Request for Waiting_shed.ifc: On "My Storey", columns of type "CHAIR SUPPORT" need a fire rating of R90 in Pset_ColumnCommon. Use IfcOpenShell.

First a look at what the model holds.

```python
import ifcopenshell
import ifcopenshell.util.element

model = ifcopenshell.open("Waiting_shed.ifc")
print(model.schema)
storey = next(s for s in model.by_type("IfcBuildingStorey") if s.Name == "My Storey")
columns = [e for e in ifcopenshell.util.element.get_decomposition(storey) if e.is_a("IfcColumn")]
seen = {}
for e in columns:
    element_type = ifcopenshell.util.element.get_type(e)
    key = (element_type.Name if element_type != e and element_type else None, ifcopenshell.util.element.get_pset(e, "Pset_ColumnCommon", "FireRating"))
    seen[key] = seen.get(key, 0) + 1
for (name, value), count in sorted(seen.items(), key=str):
    print(count, "x", name, "|", value)
```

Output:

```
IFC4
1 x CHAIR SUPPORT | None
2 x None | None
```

```python
import ifcopenshell
import ifcopenshell.api.pset
import ifcopenshell.util.element

model = ifcopenshell.open("Waiting_shed.ifc")

storey = next(s for s in model.by_type("IfcBuildingStorey") if s.Name == "My Storey")
columns = [e for e in ifcopenshell.util.element.get_decomposition(storey) if e.is_a("IfcColumn")]

count = 0
for e in columns:
    element_type = ifcopenshell.util.element.get_type(e)
    if element_type in (None, e) or element_type.Name != "CHAIR SUPPORT":
        continue
    # add_pset returns the element's existing set when there is one.
    pset = ifcopenshell.api.pset.add_pset(model, product=e, name="Pset_ColumnCommon")
    ifcopenshell.api.pset.edit_pset(model, pset=pset, properties={"FireRating": "R90"})
    count += 1

print(count, "columns updated")

model.write("Waiting_shed_v2.ifc")
```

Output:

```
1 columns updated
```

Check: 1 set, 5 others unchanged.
